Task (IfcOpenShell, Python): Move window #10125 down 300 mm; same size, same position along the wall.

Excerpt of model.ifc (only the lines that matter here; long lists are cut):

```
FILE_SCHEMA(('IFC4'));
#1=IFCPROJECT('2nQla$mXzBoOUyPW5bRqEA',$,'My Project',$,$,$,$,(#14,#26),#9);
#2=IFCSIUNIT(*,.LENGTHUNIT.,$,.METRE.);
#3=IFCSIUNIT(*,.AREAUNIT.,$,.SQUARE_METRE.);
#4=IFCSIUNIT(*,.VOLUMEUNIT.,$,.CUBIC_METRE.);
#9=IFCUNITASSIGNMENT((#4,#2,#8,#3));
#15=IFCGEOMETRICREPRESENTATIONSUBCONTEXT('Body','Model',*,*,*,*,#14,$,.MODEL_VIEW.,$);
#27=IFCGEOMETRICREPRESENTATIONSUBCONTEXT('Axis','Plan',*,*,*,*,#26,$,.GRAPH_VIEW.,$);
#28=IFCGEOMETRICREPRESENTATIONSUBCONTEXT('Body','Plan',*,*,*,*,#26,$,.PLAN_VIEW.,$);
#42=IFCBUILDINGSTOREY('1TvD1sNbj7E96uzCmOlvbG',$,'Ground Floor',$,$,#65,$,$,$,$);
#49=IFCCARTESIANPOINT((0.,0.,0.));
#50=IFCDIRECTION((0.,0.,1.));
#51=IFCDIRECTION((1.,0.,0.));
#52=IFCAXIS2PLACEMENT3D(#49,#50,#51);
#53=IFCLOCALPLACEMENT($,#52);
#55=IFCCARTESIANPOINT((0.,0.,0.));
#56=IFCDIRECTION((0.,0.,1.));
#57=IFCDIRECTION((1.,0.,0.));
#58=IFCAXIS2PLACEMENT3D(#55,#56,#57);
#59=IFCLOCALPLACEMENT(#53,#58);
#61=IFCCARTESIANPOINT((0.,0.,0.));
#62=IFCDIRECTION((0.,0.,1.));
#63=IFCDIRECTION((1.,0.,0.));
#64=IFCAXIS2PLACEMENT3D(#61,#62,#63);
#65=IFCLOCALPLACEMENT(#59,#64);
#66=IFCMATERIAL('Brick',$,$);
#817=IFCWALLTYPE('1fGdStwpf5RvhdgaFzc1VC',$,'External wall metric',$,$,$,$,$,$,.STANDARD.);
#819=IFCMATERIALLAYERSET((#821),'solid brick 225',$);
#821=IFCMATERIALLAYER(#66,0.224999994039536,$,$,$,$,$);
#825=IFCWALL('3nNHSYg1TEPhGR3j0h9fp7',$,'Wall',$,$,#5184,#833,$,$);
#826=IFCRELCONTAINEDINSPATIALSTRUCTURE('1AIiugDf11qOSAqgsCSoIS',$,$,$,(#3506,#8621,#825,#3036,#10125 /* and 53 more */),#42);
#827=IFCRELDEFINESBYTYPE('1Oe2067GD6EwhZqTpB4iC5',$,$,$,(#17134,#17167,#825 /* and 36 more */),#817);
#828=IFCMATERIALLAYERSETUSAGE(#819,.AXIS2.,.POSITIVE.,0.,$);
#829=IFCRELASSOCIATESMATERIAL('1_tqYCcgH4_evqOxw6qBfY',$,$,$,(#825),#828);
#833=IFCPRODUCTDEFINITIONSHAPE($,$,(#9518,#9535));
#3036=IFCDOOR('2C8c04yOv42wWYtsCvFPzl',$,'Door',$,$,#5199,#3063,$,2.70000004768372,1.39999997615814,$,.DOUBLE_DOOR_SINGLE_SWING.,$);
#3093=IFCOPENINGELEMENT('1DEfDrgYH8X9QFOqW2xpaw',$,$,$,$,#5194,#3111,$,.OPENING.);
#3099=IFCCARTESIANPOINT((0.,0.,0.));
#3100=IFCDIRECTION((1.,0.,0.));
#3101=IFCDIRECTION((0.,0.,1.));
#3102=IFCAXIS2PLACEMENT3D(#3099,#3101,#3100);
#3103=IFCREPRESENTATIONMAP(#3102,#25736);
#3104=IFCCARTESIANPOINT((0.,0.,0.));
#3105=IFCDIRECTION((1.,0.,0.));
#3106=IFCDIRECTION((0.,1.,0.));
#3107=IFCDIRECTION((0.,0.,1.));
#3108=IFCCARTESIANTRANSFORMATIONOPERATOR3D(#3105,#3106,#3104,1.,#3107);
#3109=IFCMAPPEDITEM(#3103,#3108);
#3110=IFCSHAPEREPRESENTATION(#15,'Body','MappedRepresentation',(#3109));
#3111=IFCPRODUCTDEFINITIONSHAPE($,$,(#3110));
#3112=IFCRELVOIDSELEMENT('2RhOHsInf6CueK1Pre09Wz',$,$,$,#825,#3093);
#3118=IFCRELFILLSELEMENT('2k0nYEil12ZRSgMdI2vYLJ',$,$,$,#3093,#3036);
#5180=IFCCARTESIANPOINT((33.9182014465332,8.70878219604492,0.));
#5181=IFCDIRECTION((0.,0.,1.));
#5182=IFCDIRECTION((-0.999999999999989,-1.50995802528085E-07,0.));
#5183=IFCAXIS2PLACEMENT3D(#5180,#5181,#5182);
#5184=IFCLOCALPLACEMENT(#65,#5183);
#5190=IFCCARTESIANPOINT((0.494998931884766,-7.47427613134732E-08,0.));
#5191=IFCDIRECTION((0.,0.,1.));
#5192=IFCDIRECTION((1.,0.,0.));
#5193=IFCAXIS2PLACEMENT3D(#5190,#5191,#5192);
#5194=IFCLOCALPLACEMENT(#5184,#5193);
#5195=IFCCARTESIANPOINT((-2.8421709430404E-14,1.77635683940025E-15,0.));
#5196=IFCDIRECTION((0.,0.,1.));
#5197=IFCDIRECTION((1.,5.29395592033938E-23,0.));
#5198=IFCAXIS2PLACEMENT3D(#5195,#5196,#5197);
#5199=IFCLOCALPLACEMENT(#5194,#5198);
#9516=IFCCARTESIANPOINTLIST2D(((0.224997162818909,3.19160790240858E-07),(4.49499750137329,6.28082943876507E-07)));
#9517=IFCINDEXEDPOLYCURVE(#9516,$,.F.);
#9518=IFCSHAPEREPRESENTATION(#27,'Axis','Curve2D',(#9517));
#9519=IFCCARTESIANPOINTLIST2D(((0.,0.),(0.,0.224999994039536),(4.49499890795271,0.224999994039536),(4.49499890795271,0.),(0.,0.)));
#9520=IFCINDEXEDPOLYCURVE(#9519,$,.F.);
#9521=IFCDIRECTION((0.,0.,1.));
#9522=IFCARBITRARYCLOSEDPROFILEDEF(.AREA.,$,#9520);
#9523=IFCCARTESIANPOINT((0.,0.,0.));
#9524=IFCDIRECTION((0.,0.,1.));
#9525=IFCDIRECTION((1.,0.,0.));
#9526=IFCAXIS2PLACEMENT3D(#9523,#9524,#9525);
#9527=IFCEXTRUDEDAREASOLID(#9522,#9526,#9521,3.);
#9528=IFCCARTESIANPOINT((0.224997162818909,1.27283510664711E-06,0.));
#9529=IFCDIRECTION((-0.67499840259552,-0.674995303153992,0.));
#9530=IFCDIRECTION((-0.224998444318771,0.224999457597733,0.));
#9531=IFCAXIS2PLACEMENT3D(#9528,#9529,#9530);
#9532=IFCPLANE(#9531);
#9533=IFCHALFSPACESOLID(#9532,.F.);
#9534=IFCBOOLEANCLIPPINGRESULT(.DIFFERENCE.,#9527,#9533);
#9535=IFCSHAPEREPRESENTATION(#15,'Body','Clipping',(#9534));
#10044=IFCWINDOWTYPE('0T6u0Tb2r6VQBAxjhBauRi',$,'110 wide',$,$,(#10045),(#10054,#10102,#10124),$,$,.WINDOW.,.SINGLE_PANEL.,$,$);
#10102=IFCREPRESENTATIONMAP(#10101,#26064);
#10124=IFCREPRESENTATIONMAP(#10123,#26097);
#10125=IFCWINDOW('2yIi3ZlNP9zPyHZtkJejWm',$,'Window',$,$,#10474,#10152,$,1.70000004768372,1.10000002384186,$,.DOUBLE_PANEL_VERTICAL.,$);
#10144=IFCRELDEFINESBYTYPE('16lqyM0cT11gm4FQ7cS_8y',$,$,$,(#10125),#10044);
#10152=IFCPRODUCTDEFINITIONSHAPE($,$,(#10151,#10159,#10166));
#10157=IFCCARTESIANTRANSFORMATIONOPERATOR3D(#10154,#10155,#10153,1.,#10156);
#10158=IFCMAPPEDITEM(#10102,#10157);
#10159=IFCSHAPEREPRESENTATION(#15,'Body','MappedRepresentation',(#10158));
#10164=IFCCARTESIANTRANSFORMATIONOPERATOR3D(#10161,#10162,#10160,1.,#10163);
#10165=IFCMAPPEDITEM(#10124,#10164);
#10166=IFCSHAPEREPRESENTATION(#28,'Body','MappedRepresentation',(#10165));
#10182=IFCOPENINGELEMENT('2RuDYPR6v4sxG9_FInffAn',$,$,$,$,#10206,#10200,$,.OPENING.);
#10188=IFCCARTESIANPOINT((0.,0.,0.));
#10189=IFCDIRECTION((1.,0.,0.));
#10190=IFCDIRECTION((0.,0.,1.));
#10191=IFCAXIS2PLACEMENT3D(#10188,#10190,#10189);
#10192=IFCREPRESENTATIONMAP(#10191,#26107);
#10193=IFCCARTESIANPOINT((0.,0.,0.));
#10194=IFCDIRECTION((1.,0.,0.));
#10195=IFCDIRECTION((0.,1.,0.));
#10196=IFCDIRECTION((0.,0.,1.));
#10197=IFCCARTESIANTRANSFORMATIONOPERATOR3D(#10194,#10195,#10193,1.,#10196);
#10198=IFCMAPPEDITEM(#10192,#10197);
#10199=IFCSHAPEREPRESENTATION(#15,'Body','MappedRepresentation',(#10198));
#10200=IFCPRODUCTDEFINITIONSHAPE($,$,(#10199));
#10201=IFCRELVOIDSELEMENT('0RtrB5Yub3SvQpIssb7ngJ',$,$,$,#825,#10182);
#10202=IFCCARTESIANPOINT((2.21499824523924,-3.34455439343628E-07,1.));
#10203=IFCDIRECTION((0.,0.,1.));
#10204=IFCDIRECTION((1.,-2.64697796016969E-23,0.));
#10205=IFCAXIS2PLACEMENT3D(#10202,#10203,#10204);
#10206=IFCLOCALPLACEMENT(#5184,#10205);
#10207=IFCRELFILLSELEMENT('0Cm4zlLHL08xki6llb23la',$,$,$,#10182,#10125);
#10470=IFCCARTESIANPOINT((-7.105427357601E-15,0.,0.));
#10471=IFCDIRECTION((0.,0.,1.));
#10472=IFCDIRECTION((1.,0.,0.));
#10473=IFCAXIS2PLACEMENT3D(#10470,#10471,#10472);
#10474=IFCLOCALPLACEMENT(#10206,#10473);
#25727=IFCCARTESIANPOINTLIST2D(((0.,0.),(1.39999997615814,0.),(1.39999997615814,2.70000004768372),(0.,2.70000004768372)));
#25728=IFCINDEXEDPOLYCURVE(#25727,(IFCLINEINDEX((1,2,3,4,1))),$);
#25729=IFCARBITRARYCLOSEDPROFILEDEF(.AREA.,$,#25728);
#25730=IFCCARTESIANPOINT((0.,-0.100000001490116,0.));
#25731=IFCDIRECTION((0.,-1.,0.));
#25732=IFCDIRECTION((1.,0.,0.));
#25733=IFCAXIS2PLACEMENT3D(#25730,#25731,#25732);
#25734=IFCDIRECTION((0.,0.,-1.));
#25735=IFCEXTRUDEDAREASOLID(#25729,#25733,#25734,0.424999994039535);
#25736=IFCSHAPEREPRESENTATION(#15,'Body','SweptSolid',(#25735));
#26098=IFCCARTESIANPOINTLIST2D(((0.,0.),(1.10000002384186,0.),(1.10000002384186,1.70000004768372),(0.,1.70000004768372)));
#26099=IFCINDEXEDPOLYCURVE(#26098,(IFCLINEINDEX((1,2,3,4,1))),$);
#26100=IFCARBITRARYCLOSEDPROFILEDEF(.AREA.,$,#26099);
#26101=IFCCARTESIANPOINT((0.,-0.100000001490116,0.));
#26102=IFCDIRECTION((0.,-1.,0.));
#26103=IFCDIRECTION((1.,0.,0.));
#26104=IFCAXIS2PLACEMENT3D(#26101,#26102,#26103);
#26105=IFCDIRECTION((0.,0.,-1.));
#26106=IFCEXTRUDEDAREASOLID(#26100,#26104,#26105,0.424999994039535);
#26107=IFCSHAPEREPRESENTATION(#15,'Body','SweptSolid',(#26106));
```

```python
import numpy as np
import ifcopenshell
import ifcopenshell.api.geometry
import ifcopenshell.util.placement
import ifcopenshell.util.unit

model = ifcopenshell.open("model.ifc")
unit_scale = ifcopenshell.util.unit.calculate_unit_scale(model)

window = model.by_guid("2yIi3ZlNP9zPyHZtkJejWm")
opening = window.FillsVoids[0].RelatingOpeningElement
dz = -0.3

shift = np.array([0.0, 0.0, dz])
# The window is placed relative to its opening, so it follows when the opening moves.
matrix = ifcopenshell.util.placement.get_local_placement(opening.ObjectPlacement)
matrix[:3, 3] += shift
ifcopenshell.api.geometry.edit_object_placement(
    model, product=opening, matrix=matrix, is_si=False, should_transform_children=True
)

print(f"moved by {dz * unit_scale:+.3f} m")

model.write("model_updated.ifc")
```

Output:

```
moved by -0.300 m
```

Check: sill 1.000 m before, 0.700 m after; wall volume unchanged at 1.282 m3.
